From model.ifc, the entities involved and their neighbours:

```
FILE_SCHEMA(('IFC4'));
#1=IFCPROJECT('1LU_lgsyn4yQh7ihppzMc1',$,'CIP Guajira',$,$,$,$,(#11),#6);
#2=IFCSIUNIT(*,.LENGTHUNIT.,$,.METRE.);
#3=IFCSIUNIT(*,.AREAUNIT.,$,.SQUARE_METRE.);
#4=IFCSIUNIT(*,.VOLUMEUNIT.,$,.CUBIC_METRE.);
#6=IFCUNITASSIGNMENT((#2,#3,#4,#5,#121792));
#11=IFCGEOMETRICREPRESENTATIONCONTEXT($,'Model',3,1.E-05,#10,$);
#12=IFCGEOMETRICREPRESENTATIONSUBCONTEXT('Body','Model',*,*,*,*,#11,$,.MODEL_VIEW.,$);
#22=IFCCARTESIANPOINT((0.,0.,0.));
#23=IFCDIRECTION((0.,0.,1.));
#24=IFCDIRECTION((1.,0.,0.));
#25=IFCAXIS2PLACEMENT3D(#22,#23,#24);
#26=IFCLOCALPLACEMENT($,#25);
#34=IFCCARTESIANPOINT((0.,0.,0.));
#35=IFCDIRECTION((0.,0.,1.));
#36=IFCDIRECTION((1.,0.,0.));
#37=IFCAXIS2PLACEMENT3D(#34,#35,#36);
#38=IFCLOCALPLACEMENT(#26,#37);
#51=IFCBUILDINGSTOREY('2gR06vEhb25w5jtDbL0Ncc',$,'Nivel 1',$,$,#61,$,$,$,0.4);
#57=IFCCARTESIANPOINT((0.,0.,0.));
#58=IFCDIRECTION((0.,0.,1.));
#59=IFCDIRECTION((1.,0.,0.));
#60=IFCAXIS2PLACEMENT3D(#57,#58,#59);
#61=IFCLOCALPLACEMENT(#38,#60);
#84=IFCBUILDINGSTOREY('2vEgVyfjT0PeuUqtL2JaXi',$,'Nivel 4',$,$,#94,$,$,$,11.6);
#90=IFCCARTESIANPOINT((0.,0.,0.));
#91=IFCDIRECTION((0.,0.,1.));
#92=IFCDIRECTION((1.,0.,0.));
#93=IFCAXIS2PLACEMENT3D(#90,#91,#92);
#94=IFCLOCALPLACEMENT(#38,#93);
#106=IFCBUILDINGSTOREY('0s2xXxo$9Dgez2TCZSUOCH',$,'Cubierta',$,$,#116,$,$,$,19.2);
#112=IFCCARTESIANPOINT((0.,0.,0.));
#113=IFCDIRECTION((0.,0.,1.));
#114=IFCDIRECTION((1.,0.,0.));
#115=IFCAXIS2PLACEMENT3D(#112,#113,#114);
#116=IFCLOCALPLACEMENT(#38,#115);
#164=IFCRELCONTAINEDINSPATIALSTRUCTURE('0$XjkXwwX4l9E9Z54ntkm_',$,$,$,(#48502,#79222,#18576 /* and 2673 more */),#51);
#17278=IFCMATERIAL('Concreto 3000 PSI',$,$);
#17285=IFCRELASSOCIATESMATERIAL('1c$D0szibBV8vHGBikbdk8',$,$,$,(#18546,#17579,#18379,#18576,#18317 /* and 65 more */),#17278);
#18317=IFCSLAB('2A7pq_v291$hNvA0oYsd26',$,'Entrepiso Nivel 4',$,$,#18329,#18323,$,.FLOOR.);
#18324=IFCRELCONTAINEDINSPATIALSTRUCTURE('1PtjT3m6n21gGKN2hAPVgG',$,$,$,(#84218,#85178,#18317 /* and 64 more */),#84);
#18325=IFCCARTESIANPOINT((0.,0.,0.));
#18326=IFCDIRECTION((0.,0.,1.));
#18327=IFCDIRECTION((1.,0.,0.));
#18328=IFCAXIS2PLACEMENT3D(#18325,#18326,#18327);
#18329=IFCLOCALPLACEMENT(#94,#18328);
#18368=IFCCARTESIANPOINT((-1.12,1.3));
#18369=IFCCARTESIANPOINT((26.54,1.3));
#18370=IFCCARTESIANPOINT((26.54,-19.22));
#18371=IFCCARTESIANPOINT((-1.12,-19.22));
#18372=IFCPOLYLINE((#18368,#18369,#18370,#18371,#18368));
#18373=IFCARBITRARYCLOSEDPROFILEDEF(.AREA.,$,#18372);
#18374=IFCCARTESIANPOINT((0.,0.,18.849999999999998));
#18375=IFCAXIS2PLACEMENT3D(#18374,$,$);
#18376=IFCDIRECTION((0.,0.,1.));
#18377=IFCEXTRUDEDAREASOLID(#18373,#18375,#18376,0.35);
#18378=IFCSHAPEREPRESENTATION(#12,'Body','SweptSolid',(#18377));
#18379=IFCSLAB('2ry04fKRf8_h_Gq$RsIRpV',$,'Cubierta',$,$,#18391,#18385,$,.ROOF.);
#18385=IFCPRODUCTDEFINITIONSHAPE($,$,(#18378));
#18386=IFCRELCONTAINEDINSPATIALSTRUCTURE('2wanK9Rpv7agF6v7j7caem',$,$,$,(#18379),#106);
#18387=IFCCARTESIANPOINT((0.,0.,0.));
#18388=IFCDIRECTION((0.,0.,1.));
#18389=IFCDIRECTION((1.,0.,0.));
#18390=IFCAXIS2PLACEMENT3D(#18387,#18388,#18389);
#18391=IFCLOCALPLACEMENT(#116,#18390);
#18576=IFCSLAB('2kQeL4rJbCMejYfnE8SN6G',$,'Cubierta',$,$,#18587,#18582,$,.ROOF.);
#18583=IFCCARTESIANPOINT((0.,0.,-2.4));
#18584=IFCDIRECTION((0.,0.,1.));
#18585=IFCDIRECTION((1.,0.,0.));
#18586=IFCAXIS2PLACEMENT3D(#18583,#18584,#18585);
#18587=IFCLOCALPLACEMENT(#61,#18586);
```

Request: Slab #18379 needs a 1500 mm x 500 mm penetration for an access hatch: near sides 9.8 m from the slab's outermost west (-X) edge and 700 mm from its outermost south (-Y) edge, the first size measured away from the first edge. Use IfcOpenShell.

```python
import numpy as np
import ifcopenshell
import ifcopenshell.api.feature
import ifcopenshell.api.geometry
import ifcopenshell.api.root
import ifcopenshell.geom
import ifcopenshell.util.placement
import ifcopenshell.util.representation
import ifcopenshell.util.shape
import ifcopenshell.util.unit

model = ifcopenshell.open("model.ifc")
unit_scale = ifcopenshell.util.unit.calculate_unit_scale(model)
settings = ifcopenshell.geom.settings()


def volume(element):
    """Net volume in cubic metres, openings subtracted."""
    shape = ifcopenshell.geom.create_shape(settings, element)
    return ifcopenshell.util.shape.get_volume(shape.geometry)


slab = model.by_guid("2ry04fKRf8_h_Gq$RsIRpV")
before = volume(slab)

# Extent in the slab's own axes, in metres. The edges named are its -X and -Y sides.
slab_shape = ifcopenshell.geom.create_shape(settings, slab)
vertices = ifcopenshell.util.shape.get_vertices(slab_shape.geometry)
x_min, y_min, bottom = vertices.min(axis=0)
top = vertices[:, 2].max()

opening = ifcopenshell.api.root.create_entity(model, ifc_class="IfcOpeningElement", name="Access hatch opening", predefined_type="OPENING")
context = ifcopenshell.util.representation.get_context(model, "Model", "Body", "MODEL_VIEW")
width, depth = 1.5, 0.5
outline = [(0.0, 0.0), (width, 0.0), (width, depth), (0.0, depth), (0.0, 0.0)]
# Overshoot both faces by 50 mm so the cut is clean.
shape = ifcopenshell.api.geometry.add_slab_representation(
    model, context=context, depth=top - bottom + 0.1, polyline=outline
)
ifcopenshell.api.geometry.assign_representation(model, product=opening, representation=shape)

matrix = ifcopenshell.util.placement.get_local_placement(slab.ObjectPlacement)
matrix[:, 3] = matrix @ np.append(np.array([x_min + 9.8, y_min + 0.7, bottom - 0.05]) / unit_scale, 1.0)
ifcopenshell.api.geometry.edit_object_placement(model, product=opening, matrix=matrix, is_si=False)
ifcopenshell.api.feature.add_feature(model, feature=opening, element=slab)

after = volume(slab)

print(f"slab volume {before:.3f} -> {after:.3f} m3")

model.write("model_rev.ifc")
```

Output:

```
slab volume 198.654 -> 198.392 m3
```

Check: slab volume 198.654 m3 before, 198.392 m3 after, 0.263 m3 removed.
